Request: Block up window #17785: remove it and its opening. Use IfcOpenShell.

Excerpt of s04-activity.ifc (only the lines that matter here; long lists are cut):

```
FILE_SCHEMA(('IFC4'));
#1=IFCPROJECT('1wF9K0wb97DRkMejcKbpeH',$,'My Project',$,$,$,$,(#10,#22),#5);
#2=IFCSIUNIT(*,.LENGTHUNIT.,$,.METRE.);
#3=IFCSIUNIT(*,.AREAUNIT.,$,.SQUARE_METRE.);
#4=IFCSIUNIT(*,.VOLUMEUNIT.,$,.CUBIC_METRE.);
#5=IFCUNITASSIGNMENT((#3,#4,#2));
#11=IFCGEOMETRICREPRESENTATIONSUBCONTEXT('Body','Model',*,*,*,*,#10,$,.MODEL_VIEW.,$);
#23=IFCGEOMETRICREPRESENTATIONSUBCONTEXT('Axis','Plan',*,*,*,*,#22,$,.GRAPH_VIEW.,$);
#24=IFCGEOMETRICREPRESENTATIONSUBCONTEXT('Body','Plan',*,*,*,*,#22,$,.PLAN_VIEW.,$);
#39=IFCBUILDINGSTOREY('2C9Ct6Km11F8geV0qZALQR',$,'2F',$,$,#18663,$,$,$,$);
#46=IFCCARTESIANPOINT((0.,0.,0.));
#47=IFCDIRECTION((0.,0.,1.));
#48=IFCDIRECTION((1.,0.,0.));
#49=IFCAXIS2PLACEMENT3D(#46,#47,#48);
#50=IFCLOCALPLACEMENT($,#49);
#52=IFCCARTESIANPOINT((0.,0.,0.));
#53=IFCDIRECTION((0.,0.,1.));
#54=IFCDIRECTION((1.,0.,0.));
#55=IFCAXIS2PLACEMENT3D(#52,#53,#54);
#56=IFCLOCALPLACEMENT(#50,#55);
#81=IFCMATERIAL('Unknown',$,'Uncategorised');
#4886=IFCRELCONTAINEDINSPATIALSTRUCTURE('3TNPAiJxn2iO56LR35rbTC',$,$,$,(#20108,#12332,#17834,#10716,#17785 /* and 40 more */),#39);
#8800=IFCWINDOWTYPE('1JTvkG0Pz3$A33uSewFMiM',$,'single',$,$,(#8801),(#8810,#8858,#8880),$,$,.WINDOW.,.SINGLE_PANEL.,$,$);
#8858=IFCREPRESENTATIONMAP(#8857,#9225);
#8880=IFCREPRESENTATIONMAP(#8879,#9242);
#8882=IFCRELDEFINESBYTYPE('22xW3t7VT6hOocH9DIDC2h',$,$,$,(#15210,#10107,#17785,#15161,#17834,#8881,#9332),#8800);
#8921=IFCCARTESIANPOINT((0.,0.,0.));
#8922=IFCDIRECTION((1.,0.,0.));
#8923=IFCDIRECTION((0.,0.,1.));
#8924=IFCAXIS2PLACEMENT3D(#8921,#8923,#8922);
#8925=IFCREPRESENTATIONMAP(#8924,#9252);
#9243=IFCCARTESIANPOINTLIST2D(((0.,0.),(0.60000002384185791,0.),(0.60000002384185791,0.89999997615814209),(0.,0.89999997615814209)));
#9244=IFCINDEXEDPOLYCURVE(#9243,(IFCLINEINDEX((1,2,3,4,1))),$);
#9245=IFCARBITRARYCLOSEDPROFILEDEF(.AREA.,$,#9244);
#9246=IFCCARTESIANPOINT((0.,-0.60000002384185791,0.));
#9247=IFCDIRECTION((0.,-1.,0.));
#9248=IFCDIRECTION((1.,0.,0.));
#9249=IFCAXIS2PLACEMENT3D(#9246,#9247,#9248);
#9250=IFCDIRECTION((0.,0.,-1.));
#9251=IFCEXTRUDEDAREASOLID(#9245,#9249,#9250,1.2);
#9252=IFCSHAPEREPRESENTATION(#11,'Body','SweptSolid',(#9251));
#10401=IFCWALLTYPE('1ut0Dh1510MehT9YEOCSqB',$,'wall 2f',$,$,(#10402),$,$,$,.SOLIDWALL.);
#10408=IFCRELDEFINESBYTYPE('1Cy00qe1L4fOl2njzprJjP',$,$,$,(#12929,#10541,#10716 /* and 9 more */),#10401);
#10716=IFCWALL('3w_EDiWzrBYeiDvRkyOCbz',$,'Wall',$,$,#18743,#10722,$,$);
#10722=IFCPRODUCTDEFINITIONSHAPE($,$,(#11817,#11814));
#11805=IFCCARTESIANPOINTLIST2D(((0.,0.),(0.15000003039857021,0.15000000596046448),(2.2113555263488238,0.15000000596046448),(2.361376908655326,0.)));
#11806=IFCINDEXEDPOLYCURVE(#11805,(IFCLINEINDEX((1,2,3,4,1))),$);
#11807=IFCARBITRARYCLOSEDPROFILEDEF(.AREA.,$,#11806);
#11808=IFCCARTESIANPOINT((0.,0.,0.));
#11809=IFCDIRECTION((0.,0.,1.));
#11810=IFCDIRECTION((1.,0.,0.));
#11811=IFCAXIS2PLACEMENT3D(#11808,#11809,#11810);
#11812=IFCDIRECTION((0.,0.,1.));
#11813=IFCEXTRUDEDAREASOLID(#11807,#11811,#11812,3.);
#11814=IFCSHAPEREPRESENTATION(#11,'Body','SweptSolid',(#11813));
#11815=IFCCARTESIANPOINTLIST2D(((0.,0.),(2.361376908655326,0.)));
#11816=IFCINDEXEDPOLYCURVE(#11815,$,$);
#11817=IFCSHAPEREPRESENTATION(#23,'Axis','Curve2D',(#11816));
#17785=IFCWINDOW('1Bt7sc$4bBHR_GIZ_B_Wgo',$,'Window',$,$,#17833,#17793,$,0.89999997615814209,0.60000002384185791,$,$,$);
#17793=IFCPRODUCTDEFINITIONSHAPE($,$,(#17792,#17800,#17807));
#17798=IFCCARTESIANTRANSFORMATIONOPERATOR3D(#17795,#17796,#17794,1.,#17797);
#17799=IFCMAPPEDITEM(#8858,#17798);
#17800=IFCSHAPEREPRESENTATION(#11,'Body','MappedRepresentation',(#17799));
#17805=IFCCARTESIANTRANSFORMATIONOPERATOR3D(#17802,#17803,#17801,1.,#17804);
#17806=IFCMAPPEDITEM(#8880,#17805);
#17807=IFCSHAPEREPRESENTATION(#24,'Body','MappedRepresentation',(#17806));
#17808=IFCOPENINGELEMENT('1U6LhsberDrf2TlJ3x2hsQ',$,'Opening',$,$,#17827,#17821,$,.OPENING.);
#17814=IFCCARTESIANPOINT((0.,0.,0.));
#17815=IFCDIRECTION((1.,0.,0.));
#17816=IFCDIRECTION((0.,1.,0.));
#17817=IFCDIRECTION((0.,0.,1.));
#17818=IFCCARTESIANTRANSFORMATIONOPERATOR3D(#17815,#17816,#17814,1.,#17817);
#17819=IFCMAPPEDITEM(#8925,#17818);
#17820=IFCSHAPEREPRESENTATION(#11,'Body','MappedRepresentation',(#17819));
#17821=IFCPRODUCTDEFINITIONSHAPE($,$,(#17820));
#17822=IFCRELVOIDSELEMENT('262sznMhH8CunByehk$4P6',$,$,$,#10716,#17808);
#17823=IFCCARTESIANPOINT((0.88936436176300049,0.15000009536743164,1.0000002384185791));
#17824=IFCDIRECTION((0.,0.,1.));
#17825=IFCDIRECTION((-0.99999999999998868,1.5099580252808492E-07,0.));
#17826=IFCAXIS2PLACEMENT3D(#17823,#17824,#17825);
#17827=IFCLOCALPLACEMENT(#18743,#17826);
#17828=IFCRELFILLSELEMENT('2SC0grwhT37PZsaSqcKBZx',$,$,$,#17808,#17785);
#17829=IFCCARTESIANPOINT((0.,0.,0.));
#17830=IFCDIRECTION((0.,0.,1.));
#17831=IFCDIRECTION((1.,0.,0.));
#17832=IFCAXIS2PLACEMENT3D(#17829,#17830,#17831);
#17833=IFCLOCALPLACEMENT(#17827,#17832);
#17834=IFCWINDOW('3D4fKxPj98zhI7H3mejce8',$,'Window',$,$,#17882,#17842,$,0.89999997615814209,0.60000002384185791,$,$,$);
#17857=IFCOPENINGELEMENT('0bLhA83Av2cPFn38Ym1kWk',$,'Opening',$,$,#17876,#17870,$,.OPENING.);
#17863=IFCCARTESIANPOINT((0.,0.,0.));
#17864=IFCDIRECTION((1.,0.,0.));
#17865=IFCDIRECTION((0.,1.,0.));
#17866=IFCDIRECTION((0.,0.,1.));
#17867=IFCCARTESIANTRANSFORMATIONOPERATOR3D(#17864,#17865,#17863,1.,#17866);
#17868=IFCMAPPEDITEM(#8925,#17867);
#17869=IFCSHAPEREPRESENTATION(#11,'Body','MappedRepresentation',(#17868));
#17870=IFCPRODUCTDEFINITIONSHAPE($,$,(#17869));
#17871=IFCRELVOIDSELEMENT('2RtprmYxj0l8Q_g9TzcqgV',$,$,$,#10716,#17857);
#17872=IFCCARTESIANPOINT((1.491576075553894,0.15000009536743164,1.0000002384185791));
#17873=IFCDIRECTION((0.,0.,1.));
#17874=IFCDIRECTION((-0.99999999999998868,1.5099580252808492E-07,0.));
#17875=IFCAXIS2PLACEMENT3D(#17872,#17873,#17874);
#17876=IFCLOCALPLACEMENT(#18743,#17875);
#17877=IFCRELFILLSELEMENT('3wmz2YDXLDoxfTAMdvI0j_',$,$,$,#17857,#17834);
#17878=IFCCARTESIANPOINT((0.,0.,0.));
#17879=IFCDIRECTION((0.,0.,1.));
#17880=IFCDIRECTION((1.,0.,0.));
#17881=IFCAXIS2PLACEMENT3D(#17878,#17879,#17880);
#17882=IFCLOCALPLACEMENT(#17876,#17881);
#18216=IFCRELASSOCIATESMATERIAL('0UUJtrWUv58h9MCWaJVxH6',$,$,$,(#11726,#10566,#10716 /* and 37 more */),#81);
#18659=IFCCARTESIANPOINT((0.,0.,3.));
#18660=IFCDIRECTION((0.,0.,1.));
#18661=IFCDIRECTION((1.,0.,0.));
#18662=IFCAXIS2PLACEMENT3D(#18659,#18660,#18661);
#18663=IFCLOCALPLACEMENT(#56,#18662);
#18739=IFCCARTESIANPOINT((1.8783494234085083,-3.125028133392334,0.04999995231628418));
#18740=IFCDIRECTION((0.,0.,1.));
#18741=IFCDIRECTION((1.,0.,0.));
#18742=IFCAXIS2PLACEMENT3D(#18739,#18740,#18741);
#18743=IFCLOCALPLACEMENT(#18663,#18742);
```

```python
import ifcopenshell
import ifcopenshell.api.feature
import ifcopenshell.api.root
import ifcopenshell.geom
import ifcopenshell.util.shape

model = ifcopenshell.open("s04-activity.ifc")
settings = ifcopenshell.geom.settings()


def volume(element):
    """Net volume in cubic metres, openings subtracted."""
    shape = ifcopenshell.geom.create_shape(settings, element)
    return ifcopenshell.util.shape.get_volume(shape.geometry)


window = model.by_guid("1Bt7sc$4bBHR_GIZ_B_Wgo")
opening = window.FillsVoids[0].RelatingOpeningElement
wall = opening.VoidsElements[0].RelatingBuildingElement
before = volume(wall)

ifcopenshell.api.root.remove_product(model, product=window)
ifcopenshell.api.feature.remove_feature(model, feature=opening)

after = volume(wall)

print(f"wall volume {before:.3f} -> {after:.3f} m3")

model.write("s04-activity_updated.ifc")
```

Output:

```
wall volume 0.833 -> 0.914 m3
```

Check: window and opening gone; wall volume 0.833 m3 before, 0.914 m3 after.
